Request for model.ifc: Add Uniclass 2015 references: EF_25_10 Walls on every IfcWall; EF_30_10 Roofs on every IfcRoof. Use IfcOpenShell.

First a look at what the model holds.

```python
import ifcopenshell

model = ifcopenshell.open("model.ifc")
print(model.schema)
print("classifications:", [c.Name for c in model.by_type("IfcClassification")])
for ifc_class in ("IfcDoor", "IfcRoof", "IfcStair", "IfcWall", "IfcWindow"):
    print(ifc_class, len(model.by_type(ifc_class)))
```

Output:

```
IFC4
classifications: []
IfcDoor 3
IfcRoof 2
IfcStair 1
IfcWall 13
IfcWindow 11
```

```python
import ifcopenshell
import ifcopenshell.api.classification

model = ifcopenshell.open("model.ifc")

system = ifcopenshell.api.classification.add_classification(model, classification="Uniclass 2015")

codes = {
    "IfcWall": ("EF_25_10", "Walls"),
    "IfcRoof": ("EF_30_10", "Roofs"),
}
for ifc_class, (code, name) in codes.items():
    products = model.by_type(ifc_class)
    ifcopenshell.api.classification.add_reference(
        model, products=products, classification=system, identification=code, name=name
    )
    print(code, len(products))

model.write("model_edited.ifc")
```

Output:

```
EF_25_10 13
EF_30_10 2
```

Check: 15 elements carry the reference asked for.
